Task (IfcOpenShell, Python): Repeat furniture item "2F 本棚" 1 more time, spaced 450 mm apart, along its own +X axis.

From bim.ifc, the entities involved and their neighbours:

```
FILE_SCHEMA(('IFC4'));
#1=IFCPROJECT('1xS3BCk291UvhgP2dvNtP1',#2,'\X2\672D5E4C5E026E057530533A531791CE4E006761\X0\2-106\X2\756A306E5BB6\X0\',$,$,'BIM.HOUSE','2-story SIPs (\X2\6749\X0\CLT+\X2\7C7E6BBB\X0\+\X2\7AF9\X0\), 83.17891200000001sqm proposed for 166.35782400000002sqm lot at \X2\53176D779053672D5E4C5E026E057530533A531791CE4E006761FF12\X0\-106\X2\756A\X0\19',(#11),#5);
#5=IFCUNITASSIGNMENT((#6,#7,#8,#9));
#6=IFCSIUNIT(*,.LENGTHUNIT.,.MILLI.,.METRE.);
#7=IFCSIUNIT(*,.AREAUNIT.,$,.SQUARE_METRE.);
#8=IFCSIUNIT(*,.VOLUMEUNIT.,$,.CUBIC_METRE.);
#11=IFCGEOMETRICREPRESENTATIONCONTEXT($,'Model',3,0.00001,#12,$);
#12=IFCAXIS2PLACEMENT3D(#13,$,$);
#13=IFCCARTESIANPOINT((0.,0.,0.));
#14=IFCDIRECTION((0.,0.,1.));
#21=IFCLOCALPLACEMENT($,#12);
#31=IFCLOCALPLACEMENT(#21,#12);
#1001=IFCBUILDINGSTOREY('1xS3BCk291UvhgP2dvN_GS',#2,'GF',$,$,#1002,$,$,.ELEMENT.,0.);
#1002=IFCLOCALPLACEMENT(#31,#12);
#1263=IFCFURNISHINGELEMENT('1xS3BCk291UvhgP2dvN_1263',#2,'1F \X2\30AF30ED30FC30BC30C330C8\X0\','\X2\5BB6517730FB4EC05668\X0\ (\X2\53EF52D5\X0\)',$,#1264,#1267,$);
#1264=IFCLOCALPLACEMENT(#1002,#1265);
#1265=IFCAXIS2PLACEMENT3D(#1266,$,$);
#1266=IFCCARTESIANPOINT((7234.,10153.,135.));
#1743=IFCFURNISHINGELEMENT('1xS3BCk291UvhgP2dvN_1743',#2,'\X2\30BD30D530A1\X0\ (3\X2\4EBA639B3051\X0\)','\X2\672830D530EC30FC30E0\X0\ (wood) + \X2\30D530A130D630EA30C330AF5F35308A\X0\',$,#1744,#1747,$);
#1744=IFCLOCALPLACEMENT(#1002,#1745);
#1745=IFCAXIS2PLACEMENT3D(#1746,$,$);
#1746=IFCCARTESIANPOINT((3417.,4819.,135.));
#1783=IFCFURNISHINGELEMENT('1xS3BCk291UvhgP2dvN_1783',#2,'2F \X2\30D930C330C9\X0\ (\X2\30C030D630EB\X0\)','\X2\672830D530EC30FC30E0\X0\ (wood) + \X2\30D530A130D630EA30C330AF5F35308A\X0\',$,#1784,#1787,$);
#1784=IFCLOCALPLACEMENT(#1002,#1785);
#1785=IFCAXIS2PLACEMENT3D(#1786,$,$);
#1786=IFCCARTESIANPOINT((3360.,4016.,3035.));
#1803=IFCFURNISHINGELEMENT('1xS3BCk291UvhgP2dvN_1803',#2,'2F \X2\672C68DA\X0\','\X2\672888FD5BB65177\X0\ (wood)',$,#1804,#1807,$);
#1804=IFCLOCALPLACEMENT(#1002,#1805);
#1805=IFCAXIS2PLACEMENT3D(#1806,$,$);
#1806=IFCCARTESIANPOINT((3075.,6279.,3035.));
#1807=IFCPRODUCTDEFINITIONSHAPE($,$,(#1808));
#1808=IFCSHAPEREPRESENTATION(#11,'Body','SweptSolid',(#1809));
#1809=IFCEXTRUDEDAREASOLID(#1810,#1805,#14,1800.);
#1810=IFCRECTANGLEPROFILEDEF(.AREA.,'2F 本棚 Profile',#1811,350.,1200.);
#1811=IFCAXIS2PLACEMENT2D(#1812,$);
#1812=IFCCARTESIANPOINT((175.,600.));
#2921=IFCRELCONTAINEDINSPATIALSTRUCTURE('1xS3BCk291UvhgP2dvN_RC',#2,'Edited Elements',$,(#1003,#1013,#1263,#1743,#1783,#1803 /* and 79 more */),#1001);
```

```python
import ifcopenshell
import ifcopenshell.api.geometry
import ifcopenshell.api.root
import ifcopenshell.util.element
import ifcopenshell.util.placement
import ifcopenshell.util.unit

model = ifcopenshell.open("bim.ifc")
unit_scale = ifcopenshell.util.unit.calculate_unit_scale(model)


def reuse_history(source, copy):
    """copy_class also copies each property set's owner history, people and application; keep the originals."""
    for rel in copy.IsDefinedBy:
        if rel.is_a("IfcRelDefinesByProperties") and (history := rel.RelatingPropertyDefinition.OwnerHistory):
            rel.RelatingPropertyDefinition.OwnerHistory = source.OwnerHistory
            ifcopenshell.util.element.remove_deep2(model, history)


source = model.by_id(1803)
base = ifcopenshell.util.placement.get_local_placement(source.ObjectPlacement)
step = base[:3, 0] * 0.45 / unit_scale

for i in range(1, 2):
    copy = ifcopenshell.api.root.copy_class(model, product=source)
    copy.Representation = ifcopenshell.util.element.copy_deep(
        model, source.Representation, exclude=["IfcGeometricRepresentationContext", "IfcRepresentationMap"]
    )
    reuse_history(source, copy)
    matrix = base.copy()
    matrix[:3, 3] += i * step
    print("added at", matrix[:3, 3].round(3) + 0.0)
    ifcopenshell.api.geometry.edit_object_placement(model, product=copy, matrix=matrix, is_si=False)

model.write("bim-out.ifc")
```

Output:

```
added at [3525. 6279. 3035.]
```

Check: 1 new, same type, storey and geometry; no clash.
